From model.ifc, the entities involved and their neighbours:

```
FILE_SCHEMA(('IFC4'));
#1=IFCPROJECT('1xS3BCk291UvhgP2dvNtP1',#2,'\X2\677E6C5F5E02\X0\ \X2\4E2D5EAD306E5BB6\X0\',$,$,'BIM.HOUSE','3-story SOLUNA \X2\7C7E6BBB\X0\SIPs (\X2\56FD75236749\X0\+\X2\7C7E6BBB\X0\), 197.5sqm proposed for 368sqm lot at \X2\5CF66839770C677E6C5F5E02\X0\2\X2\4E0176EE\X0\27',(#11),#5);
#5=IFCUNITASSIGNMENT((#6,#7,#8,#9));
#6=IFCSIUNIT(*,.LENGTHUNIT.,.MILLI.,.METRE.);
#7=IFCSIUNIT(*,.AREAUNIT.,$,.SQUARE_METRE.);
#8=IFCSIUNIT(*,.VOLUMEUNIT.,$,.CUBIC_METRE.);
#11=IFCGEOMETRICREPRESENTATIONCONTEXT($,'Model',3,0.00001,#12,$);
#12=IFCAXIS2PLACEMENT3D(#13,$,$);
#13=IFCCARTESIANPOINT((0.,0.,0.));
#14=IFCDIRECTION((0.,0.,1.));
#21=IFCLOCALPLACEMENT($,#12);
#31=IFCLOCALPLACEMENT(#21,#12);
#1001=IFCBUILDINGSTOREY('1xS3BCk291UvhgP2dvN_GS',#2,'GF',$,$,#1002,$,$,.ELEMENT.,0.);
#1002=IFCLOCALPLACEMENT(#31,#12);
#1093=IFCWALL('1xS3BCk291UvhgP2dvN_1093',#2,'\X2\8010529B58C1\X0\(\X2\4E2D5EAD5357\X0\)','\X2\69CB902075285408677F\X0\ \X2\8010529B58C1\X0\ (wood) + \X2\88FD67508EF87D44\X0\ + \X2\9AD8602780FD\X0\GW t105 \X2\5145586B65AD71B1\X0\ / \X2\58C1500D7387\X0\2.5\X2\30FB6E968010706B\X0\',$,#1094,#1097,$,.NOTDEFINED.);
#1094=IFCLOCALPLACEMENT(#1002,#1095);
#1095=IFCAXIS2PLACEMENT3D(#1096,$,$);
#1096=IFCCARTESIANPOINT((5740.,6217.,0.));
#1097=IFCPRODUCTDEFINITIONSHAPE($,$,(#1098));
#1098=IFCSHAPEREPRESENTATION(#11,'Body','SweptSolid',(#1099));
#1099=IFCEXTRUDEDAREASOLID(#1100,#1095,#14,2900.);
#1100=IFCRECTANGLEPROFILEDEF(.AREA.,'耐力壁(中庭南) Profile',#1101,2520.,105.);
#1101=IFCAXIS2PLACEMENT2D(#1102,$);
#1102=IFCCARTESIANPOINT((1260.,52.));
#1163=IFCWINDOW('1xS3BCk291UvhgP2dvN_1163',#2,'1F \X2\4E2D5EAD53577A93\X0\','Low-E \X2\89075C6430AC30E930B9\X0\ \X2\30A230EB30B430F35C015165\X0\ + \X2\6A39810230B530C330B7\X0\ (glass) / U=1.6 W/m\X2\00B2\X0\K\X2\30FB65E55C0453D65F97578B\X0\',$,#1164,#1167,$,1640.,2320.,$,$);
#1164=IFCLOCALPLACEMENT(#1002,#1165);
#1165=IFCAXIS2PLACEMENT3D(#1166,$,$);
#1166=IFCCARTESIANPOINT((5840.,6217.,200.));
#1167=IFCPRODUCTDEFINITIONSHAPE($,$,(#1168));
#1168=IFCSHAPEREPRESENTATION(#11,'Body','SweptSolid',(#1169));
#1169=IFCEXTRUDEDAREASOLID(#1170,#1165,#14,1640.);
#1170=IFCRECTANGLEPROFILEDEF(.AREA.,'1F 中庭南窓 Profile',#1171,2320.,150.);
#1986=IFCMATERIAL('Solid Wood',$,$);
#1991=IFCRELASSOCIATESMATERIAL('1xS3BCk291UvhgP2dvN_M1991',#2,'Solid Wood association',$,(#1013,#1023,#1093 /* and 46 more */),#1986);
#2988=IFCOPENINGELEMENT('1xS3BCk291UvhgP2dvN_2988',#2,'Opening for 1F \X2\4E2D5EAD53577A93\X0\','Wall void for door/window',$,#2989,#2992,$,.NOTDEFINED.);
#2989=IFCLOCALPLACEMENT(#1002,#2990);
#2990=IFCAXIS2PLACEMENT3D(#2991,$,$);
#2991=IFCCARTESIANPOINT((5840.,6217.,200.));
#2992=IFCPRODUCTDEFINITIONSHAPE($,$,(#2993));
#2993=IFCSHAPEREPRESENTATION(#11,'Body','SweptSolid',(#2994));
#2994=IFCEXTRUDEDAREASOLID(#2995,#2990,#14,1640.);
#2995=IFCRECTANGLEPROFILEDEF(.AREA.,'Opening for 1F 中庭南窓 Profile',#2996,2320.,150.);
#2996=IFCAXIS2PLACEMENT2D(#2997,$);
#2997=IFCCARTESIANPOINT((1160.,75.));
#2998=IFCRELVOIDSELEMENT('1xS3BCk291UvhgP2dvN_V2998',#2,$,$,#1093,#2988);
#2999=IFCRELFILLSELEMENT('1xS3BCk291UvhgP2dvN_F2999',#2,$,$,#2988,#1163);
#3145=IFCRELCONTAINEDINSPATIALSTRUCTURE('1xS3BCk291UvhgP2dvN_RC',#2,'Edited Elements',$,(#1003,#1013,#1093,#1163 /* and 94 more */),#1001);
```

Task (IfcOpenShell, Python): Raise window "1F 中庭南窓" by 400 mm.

```python
import numpy as np
import ifcopenshell
import ifcopenshell.api.geometry
import ifcopenshell.util.placement
import ifcopenshell.util.unit

model = ifcopenshell.open("model.ifc")
unit_scale = ifcopenshell.util.unit.calculate_unit_scale(model)

window = model.by_id(1163)
opening = window.FillsVoids[0].RelatingOpeningElement
dz = 0.4 / unit_scale

shift = np.array([0.0, 0.0, dz])
# The window is not placed relative to its opening, so move both.
for product in (opening, window):
    matrix = ifcopenshell.util.placement.get_local_placement(product.ObjectPlacement)
    matrix[:3, 3] += shift
    ifcopenshell.api.geometry.edit_object_placement(model, product=product, matrix=matrix, is_si=False)

print(f"moved by {dz * unit_scale:+.3f} m")

model.write("model_updated.ifc")
```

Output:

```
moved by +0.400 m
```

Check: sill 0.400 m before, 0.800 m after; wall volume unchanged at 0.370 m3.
